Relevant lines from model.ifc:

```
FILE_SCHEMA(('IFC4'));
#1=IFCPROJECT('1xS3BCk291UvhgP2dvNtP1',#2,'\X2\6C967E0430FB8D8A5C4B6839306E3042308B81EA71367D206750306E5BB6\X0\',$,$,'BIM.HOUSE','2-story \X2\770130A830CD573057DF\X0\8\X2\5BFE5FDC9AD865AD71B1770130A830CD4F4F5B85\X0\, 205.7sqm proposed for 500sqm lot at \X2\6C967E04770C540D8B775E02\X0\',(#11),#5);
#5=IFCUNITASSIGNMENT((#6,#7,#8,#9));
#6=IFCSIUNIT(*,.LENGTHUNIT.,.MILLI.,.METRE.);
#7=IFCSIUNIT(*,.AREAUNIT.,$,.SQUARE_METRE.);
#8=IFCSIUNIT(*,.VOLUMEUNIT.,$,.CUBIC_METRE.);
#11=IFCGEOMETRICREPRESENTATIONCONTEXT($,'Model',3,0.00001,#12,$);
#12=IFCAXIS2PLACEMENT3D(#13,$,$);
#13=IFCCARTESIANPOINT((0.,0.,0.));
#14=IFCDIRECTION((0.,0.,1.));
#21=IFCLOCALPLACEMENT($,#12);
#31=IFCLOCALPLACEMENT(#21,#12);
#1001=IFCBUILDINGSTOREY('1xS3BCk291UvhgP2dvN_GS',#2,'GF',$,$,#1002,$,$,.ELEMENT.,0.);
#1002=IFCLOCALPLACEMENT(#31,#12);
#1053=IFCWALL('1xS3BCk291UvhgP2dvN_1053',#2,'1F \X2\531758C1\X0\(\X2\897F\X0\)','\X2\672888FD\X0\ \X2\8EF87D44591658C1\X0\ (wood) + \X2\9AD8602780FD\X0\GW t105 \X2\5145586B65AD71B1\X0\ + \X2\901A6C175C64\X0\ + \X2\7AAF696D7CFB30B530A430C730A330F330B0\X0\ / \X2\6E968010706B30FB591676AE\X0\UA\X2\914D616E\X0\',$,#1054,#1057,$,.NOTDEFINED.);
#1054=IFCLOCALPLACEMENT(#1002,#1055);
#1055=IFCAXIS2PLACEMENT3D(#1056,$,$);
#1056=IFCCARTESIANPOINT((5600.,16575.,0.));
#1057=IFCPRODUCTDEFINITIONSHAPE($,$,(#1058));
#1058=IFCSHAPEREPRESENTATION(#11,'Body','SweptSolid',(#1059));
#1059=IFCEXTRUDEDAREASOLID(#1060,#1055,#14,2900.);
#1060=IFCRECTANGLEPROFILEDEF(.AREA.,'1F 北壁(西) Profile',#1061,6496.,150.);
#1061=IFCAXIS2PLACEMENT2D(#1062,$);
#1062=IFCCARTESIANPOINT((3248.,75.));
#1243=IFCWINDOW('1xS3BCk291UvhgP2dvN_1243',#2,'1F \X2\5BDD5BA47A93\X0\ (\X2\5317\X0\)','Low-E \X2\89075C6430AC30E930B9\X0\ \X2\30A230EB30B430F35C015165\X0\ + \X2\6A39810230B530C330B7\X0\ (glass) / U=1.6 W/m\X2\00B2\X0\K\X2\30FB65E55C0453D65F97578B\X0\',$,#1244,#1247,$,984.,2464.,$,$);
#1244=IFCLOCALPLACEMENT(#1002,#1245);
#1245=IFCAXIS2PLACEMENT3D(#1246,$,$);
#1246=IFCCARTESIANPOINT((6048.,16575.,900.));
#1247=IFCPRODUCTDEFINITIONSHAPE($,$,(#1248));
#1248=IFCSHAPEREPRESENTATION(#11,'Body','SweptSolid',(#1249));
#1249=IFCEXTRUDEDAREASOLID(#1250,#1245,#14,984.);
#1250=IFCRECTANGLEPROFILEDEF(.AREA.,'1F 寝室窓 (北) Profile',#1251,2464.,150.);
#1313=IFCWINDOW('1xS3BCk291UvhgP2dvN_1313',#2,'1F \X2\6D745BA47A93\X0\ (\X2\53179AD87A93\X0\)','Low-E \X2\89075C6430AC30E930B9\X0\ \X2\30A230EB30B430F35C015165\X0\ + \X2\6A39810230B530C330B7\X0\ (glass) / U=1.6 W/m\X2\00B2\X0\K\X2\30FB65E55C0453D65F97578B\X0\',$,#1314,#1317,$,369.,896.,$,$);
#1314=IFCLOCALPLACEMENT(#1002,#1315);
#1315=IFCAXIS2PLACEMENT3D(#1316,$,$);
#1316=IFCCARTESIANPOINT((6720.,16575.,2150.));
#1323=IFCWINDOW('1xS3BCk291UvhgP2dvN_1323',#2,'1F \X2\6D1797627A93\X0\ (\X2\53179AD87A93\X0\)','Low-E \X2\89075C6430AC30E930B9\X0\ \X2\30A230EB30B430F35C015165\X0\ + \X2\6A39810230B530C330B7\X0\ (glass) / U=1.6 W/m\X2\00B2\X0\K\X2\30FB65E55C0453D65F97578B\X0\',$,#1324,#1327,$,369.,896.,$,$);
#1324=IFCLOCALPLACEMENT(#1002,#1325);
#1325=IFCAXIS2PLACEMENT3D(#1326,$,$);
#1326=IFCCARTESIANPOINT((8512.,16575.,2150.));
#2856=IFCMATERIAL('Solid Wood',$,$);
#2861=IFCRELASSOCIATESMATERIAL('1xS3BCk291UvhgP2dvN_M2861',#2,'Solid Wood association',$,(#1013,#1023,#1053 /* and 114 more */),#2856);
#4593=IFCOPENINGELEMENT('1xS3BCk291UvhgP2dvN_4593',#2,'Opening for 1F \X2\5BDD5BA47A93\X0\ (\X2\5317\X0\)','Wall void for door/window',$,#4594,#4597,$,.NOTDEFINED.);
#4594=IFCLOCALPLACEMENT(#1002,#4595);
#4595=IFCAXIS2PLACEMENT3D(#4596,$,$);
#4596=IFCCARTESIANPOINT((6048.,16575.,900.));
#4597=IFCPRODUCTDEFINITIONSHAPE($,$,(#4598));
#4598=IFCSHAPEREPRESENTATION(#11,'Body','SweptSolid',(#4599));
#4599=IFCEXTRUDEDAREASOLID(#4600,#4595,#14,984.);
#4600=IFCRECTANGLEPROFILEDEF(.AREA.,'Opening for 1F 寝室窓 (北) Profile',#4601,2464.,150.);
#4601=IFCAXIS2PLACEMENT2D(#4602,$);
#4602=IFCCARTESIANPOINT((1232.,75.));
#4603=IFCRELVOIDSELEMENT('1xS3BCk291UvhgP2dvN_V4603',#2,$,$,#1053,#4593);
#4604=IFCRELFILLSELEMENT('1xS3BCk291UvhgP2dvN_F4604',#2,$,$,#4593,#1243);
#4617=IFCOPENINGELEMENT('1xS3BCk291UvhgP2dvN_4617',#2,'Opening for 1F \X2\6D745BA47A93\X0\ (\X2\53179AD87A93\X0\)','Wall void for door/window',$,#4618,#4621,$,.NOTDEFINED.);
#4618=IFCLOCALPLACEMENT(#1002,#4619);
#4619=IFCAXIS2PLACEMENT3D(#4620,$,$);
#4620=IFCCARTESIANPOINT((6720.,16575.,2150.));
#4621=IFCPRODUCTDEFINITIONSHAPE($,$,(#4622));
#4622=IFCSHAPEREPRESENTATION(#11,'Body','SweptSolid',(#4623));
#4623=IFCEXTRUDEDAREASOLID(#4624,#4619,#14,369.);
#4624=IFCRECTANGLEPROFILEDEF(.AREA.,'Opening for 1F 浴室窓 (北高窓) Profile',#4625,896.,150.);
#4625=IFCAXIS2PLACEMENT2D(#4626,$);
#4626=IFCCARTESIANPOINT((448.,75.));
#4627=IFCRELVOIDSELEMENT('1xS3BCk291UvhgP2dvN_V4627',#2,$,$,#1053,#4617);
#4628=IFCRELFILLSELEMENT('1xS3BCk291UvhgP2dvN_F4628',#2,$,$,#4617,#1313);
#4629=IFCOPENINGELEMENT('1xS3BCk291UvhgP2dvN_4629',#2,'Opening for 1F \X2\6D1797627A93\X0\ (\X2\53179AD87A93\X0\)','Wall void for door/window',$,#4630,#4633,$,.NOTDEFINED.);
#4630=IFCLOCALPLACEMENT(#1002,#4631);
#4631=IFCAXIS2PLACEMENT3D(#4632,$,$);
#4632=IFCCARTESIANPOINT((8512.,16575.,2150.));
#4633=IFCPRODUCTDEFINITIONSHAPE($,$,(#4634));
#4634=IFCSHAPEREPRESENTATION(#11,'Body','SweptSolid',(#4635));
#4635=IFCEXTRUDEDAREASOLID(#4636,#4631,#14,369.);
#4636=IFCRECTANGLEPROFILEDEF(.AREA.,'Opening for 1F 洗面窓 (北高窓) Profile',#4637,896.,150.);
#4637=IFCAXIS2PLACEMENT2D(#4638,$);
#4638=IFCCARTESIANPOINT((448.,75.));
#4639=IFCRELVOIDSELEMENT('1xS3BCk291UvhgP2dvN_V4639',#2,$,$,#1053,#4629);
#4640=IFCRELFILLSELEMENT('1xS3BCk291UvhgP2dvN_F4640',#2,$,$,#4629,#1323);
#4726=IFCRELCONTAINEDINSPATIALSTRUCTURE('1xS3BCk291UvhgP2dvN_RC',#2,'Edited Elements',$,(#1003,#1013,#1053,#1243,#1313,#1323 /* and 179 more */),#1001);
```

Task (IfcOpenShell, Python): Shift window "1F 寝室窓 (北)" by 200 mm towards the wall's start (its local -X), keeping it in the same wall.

```python
import ifcopenshell
import ifcopenshell.api.geometry
import ifcopenshell.util.placement

model = ifcopenshell.open("model.ifc")

window = model.by_id(1243)
opening = window.FillsVoids[0].RelatingOpeningElement
wall = opening.VoidsElements[0].RelatingBuildingElement

wall_matrix = ifcopenshell.util.placement.get_local_placement(wall.ObjectPlacement)
shift = wall_matrix[:3, 0] * -200.0
before = ifcopenshell.util.placement.get_local_placement(window.ObjectPlacement)[:3, 3].copy()

# The window is not placed relative to its opening, so move both.
for product in (opening, window):
    matrix = ifcopenshell.util.placement.get_local_placement(product.ObjectPlacement)
    matrix[:3, 3] += shift
    ifcopenshell.api.geometry.edit_object_placement(model, product=product, matrix=matrix, is_si=False)

after = ifcopenshell.util.placement.get_local_placement(window.ObjectPlacement)[:3, 3]
print("window moved by", (after - before).round(3) + 0.0)

model.write("model_rev.ifc")
```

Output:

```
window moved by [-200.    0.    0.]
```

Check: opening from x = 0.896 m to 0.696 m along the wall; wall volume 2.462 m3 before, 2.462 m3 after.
